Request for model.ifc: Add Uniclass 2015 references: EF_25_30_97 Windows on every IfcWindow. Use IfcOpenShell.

First a look at what the model holds.

```python
import ifcopenshell

model = ifcopenshell.open("model.ifc")
print(model.schema)
print("classifications:", [c.Name for c in model.by_type("IfcClassification")])
for ifc_class in ("IfcDoor", "IfcRoof", "IfcStair", "IfcWall", "IfcWindow"):
    print(ifc_class, len(model.by_type(ifc_class)))
```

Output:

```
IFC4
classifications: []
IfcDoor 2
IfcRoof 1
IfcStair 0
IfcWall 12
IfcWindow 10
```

```python
import ifcopenshell
import ifcopenshell.api.classification

model = ifcopenshell.open("model.ifc")

system = ifcopenshell.api.classification.add_classification(model, classification="Uniclass 2015")

codes = {
    "IfcWindow": ("EF_25_30_97", "Windows"),
}
for ifc_class, (code, name) in codes.items():
    products = model.by_type(ifc_class)
    ifcopenshell.api.classification.add_reference(
        model, products=products, classification=system, identification=code, name=name
    )
    print(code, len(products))

model.write("model-out.ifc")
```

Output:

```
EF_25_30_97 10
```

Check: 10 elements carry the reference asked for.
